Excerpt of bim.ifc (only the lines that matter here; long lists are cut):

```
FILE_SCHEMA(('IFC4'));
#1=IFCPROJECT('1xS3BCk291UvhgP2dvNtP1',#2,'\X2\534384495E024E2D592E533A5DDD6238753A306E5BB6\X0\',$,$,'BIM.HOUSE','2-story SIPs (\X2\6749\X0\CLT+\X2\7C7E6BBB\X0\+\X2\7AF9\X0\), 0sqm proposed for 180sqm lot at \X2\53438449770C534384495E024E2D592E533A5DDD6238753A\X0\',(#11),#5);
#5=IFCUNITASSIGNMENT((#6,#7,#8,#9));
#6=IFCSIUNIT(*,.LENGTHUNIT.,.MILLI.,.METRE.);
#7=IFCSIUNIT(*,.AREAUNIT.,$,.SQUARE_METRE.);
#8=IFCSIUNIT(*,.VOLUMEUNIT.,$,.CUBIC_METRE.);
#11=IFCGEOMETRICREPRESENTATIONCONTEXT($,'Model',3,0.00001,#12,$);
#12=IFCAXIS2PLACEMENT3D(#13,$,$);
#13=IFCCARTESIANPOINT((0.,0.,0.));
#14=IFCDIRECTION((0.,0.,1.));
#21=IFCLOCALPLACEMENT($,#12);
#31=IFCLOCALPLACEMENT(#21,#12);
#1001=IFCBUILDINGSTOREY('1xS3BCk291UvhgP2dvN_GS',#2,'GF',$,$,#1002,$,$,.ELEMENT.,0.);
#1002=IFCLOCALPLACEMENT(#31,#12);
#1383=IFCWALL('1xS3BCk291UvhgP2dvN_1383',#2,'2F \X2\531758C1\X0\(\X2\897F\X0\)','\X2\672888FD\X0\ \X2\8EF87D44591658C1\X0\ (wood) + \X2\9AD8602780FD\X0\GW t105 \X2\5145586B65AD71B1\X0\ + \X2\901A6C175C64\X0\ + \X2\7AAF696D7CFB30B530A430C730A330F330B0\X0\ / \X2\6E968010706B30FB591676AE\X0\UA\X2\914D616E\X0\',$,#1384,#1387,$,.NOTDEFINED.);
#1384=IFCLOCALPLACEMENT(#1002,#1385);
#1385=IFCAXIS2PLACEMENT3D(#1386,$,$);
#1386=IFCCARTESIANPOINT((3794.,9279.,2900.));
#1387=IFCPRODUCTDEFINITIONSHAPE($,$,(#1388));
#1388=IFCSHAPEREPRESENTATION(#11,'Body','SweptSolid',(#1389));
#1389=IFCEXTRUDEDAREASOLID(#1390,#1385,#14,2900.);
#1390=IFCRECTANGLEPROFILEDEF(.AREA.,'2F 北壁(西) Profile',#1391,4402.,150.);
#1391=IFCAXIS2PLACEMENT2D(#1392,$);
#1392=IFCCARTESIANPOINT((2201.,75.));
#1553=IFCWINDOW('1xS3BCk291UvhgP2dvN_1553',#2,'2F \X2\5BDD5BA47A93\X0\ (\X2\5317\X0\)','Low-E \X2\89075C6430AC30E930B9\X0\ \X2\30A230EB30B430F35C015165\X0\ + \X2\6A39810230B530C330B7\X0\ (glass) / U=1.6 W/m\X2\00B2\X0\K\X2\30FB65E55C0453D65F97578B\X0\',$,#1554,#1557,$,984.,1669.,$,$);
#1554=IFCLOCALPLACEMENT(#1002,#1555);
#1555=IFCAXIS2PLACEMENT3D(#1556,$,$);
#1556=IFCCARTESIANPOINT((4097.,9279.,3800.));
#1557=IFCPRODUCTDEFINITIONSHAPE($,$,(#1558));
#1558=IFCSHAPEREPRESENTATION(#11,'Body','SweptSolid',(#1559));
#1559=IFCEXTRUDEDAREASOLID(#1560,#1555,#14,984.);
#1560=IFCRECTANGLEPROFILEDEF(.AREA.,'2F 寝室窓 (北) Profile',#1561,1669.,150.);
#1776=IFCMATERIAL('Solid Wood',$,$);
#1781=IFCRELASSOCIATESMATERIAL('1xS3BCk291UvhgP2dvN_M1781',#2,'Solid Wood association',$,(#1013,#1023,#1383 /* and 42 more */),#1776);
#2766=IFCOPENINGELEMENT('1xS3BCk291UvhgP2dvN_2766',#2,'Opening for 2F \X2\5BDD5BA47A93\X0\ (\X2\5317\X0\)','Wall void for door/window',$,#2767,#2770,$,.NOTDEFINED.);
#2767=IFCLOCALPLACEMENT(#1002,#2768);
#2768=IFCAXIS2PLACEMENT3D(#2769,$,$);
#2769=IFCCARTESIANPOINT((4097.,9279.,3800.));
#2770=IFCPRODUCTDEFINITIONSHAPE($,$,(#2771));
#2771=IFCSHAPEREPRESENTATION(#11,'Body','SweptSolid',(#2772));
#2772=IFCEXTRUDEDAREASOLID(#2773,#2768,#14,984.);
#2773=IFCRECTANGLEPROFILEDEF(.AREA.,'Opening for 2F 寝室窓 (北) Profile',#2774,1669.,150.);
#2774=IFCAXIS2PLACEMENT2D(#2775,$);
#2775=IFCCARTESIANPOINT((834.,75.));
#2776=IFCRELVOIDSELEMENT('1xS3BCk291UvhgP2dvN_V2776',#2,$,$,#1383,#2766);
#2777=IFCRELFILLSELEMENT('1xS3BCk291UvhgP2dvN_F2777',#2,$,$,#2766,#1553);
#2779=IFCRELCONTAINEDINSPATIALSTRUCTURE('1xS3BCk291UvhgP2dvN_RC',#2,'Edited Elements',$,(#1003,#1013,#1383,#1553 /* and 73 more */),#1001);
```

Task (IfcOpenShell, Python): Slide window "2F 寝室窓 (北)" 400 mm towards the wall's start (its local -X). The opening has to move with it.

```python
import ifcopenshell
import ifcopenshell.api.geometry
import ifcopenshell.util.placement
import ifcopenshell.util.unit

model = ifcopenshell.open("bim.ifc")
unit_scale = ifcopenshell.util.unit.calculate_unit_scale(model)

window = model.by_guid("1xS3BCk291UvhgP2dvN_1553")
opening = window.FillsVoids[0].RelatingOpeningElement
wall = opening.VoidsElements[0].RelatingBuildingElement

wall_matrix = ifcopenshell.util.placement.get_local_placement(wall.ObjectPlacement)
shift = wall_matrix[:3, 0] * -0.4 / unit_scale
before = ifcopenshell.util.placement.get_local_placement(window.ObjectPlacement)[:3, 3].copy()

# The window is not placed relative to its opening, so move both.
for product in (opening, window):
    matrix = ifcopenshell.util.placement.get_local_placement(product.ObjectPlacement)
    matrix[:3, 3] += shift
    ifcopenshell.api.geometry.edit_object_placement(model, product=product, matrix=matrix, is_si=False)

after = ifcopenshell.util.placement.get_local_placement(window.ObjectPlacement)[:3, 3]
print("window moved by", (after - before).round(3) + 0.0)

model.write("bim_updated.ifc")
```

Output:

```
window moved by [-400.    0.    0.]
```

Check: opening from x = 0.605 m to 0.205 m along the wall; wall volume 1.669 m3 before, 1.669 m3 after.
